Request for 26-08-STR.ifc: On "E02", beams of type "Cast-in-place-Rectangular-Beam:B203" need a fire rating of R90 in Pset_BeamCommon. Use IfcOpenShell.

First a look at what the model holds.

```python
import ifcopenshell
import ifcopenshell.util.element

model = ifcopenshell.open("26-08-STR.ifc")
print(model.schema)
storey = next(s for s in model.by_type("IfcBuildingStorey") if s.Name == "E02")
beams = [e for e in ifcopenshell.util.element.get_decomposition(storey) if e.is_a("IfcBeam")]
seen = {}
for e in beams:
    element_type = ifcopenshell.util.element.get_type(e)
    key = (element_type.Name if element_type != e and element_type else None, ifcopenshell.util.element.get_pset(e, "Pset_BeamCommon", "FireRating"))
    seen[key] = seen.get(key, 0) + 1
for (name, value), count in sorted(seen.items(), key=str):
    print(count, "x", name, "|", value)
```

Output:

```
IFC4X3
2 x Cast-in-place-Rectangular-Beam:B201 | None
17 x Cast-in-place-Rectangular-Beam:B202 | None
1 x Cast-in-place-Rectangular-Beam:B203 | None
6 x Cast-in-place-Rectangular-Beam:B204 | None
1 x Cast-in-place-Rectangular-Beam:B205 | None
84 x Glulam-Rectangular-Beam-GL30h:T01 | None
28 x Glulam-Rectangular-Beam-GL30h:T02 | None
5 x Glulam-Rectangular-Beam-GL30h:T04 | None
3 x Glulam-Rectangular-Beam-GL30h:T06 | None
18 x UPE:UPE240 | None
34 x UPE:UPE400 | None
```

```python
import ifcopenshell
import ifcopenshell.api.pset
import ifcopenshell.util.element

model = ifcopenshell.open("26-08-STR.ifc")

storey = next(s for s in model.by_type("IfcBuildingStorey") if s.Name == "E02")
beams = [e for e in ifcopenshell.util.element.get_decomposition(storey) if e.is_a("IfcBeam")]

count = 0
for e in beams:
    element_type = ifcopenshell.util.element.get_type(e)
    if element_type in (None, e) or element_type.Name != "Cast-in-place-Rectangular-Beam:B203":
        continue
    # add_pset returns the element's existing set when there is one.
    pset = ifcopenshell.api.pset.add_pset(model, product=e, name="Pset_BeamCommon")
    ifcopenshell.api.pset.edit_pset(model, pset=pset, properties={"FireRating": "R90"})
    count += 1

print(count, "beams updated")

model.write("26-08-STR_rev.ifc")
```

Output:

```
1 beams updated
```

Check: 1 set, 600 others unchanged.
